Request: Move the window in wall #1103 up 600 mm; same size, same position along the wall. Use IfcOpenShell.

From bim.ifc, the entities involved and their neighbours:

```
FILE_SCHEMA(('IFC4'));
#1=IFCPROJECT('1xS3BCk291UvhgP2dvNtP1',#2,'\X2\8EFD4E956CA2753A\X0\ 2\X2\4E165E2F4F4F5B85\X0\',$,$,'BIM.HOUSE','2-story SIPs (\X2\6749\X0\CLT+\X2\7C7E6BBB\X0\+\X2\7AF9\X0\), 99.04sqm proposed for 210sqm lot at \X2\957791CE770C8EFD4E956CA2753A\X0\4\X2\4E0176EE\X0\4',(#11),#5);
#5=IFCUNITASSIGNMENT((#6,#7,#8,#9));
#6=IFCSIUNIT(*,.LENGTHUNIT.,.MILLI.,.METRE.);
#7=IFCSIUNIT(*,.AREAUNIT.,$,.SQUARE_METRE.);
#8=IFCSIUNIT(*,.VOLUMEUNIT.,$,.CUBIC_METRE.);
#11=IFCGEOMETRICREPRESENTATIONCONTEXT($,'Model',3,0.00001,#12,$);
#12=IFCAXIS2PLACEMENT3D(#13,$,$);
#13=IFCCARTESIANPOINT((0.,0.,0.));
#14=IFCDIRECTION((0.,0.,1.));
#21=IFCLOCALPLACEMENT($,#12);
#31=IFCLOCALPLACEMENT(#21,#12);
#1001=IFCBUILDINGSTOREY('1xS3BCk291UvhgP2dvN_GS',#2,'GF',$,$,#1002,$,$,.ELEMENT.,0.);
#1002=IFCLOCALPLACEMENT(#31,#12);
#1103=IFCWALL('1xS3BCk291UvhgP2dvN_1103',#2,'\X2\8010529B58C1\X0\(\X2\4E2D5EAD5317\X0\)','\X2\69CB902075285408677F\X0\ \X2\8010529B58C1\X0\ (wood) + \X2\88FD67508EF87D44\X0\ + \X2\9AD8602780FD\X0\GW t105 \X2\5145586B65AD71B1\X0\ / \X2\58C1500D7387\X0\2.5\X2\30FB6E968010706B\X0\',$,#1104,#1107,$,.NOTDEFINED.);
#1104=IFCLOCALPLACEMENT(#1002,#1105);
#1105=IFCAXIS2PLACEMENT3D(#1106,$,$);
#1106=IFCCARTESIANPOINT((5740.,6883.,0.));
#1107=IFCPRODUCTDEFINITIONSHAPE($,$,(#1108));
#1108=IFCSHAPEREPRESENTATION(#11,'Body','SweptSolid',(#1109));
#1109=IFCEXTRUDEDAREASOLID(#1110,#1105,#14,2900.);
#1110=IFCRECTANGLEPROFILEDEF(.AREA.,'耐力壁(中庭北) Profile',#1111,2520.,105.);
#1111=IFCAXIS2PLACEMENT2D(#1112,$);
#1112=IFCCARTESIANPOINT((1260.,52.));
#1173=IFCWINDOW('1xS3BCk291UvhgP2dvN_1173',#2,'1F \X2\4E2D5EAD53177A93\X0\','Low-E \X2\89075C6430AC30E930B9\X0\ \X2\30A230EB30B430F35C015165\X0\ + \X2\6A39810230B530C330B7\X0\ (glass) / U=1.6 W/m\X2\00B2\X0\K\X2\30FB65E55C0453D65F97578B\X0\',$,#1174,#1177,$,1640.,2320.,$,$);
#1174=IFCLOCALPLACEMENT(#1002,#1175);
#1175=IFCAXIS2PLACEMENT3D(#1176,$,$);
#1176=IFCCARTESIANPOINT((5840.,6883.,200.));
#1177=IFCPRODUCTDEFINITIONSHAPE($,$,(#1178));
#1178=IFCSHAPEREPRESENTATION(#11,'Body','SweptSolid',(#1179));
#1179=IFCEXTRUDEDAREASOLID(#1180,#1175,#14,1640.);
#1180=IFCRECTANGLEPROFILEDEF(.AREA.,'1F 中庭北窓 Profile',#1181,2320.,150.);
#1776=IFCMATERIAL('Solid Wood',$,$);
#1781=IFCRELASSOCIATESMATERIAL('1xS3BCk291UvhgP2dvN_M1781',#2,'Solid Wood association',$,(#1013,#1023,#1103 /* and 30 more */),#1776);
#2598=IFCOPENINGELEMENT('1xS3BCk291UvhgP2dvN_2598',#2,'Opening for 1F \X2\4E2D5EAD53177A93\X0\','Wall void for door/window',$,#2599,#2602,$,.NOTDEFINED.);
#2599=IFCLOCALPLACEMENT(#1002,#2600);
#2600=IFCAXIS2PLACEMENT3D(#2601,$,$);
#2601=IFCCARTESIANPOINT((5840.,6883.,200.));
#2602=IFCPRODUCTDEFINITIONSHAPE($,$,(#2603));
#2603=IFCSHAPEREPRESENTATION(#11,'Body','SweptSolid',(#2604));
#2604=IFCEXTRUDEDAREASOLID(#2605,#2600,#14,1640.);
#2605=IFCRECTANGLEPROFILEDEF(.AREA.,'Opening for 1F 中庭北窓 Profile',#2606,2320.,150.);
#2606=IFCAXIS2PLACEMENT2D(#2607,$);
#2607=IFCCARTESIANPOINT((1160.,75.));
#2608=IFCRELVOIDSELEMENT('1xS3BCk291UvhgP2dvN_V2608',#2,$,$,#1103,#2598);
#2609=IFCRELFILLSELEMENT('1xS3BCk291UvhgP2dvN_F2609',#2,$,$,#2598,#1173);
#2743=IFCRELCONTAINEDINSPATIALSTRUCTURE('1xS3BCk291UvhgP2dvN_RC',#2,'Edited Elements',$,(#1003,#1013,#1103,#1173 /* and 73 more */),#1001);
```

```python
import numpy as np
import ifcopenshell
import ifcopenshell.api.geometry
import ifcopenshell.util.placement
import ifcopenshell.util.unit

model = ifcopenshell.open("bim.ifc")
unit_scale = ifcopenshell.util.unit.calculate_unit_scale(model)

window = model.by_guid("1xS3BCk291UvhgP2dvN_1173")
opening = window.FillsVoids[0].RelatingOpeningElement
dz = 0.6 / unit_scale

shift = np.array([0.0, 0.0, dz])
# The window is not placed relative to its opening, so move both.
for product in (opening, window):
    matrix = ifcopenshell.util.placement.get_local_placement(product.ObjectPlacement)
    matrix[:3, 3] += shift
    ifcopenshell.api.geometry.edit_object_placement(model, product=product, matrix=matrix, is_si=False)

print(f"moved by {dz * unit_scale:+.3f} m")

model.write("bim-out.ifc")
```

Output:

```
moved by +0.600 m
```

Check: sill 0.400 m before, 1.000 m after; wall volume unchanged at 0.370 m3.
